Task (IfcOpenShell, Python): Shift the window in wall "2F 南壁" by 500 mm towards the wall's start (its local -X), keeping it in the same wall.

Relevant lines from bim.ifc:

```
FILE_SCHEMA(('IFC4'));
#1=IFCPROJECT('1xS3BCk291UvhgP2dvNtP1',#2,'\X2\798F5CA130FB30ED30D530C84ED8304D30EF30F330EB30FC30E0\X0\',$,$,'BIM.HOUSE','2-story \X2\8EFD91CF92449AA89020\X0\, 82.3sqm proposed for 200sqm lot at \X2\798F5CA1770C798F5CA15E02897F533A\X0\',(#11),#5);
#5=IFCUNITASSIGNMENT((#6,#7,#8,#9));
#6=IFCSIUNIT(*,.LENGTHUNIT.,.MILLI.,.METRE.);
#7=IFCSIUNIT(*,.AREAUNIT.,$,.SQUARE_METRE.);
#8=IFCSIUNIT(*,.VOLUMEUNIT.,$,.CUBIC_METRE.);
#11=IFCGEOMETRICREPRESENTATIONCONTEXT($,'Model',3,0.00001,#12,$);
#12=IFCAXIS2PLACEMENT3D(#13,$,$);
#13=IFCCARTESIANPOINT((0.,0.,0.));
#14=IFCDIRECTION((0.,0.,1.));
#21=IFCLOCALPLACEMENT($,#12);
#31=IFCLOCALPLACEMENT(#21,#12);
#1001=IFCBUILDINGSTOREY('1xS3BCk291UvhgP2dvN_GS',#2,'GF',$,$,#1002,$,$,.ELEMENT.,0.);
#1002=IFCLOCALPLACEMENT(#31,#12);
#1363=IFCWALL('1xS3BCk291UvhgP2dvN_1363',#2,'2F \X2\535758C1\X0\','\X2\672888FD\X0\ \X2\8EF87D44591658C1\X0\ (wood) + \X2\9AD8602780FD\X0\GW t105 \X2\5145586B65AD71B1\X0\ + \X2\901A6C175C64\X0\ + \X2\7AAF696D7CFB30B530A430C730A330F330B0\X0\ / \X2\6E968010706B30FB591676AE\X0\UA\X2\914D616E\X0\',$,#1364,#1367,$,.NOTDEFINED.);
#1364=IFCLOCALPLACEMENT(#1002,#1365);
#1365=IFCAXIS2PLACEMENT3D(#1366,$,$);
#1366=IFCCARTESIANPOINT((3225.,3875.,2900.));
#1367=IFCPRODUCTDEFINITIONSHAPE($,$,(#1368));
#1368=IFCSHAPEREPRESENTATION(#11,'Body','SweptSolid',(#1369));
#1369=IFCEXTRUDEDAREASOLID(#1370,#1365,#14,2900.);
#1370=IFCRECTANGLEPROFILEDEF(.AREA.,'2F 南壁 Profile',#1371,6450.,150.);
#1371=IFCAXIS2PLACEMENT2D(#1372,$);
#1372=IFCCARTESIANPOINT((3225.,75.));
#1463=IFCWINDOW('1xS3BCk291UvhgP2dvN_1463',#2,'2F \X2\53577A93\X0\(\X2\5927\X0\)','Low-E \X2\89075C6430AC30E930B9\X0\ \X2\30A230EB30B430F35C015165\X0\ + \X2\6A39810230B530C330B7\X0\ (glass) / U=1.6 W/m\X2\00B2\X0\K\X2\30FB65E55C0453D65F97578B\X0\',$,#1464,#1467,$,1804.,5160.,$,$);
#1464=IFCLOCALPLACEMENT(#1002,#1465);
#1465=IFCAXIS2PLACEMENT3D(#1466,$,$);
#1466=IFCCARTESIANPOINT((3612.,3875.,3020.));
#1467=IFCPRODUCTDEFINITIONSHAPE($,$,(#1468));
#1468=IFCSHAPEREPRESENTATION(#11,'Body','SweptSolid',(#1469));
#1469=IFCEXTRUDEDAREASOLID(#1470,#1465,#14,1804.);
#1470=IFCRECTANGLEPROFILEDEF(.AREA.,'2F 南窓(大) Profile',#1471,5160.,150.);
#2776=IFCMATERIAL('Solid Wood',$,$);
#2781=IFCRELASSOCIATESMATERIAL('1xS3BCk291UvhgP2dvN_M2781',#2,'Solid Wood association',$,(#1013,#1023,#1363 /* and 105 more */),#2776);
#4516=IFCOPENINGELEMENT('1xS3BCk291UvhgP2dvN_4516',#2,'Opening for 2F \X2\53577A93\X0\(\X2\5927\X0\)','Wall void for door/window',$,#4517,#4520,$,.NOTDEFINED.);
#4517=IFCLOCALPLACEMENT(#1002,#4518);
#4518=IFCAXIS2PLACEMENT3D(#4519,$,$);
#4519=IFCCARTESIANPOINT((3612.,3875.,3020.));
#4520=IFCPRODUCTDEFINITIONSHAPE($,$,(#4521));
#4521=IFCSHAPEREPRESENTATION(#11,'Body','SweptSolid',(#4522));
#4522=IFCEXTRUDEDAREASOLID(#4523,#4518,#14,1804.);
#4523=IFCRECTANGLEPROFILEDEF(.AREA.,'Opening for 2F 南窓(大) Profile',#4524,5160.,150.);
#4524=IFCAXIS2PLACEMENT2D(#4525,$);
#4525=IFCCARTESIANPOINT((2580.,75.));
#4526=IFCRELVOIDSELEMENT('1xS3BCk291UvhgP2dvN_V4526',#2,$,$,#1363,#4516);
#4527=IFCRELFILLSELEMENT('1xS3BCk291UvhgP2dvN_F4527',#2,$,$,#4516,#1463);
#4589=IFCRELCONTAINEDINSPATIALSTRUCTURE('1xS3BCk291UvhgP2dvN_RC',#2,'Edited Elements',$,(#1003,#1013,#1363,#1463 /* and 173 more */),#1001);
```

```python
import ifcopenshell
import ifcopenshell.api.geometry
import ifcopenshell.util.placement

model = ifcopenshell.open("bim.ifc")

window = model.by_id(1463)
opening = window.FillsVoids[0].RelatingOpeningElement
wall = opening.VoidsElements[0].RelatingBuildingElement

wall_matrix = ifcopenshell.util.placement.get_local_placement(wall.ObjectPlacement)
shift = wall_matrix[:3, 0] * -500.0
before = ifcopenshell.util.placement.get_local_placement(window.ObjectPlacement)[:3, 3].copy()

# The window is not placed relative to its opening, so move both.
for product in (opening, window):
    matrix = ifcopenshell.util.placement.get_local_placement(product.ObjectPlacement)
    matrix[:3, 3] += shift
    ifcopenshell.api.geometry.edit_object_placement(model, product=product, matrix=matrix, is_si=False)

after = ifcopenshell.util.placement.get_local_placement(window.ObjectPlacement)[:3, 3]
print("window moved by", (after - before).round(3) + 0.0)

model.write("bim_updated.ifc")
```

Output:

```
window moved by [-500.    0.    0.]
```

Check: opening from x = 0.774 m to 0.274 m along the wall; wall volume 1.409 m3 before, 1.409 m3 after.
